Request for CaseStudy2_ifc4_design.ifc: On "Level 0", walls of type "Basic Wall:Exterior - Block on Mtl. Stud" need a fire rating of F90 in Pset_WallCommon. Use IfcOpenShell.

First a look at what the model holds.

```python
import ifcopenshell
import ifcopenshell.util.element

model = ifcopenshell.open("CaseStudy2_ifc4_design.ifc")
print(model.schema)
storey = next(s for s in model.by_type("IfcBuildingStorey") if s.Name == "Level 0")
walls = [e for e in ifcopenshell.util.element.get_decomposition(storey) if e.is_a("IfcWall")]
seen = {}
for e in walls:
    element_type = ifcopenshell.util.element.get_type(e)
    key = (element_type.Name if element_type != e and element_type else None, ifcopenshell.util.element.get_pset(e, "Pset_WallCommon", "FireRating"))
    seen[key] = seen.get(key, 0) + 1
for (name, value), count in sorted(seen.items(), key=str):
    print(count, "x", name, "|", value)
```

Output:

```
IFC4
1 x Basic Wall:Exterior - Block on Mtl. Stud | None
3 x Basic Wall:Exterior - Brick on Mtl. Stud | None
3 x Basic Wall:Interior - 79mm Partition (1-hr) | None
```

```python
import ifcopenshell
import ifcopenshell.api.pset
import ifcopenshell.util.element

model = ifcopenshell.open("CaseStudy2_ifc4_design.ifc")

storey = next(s for s in model.by_type("IfcBuildingStorey") if s.Name == "Level 0")
walls = [e for e in ifcopenshell.util.element.get_decomposition(storey) if e.is_a("IfcWall")]

count = 0
for e in walls:
    element_type = ifcopenshell.util.element.get_type(e)
    if element_type in (None, e) or element_type.Name != "Basic Wall:Exterior - Block on Mtl. Stud":
        continue
    # add_pset returns the element's existing set when there is one.
    pset = ifcopenshell.api.pset.add_pset(model, product=e, name="Pset_WallCommon")
    ifcopenshell.api.pset.edit_pset(model, pset=pset, properties={"FireRating": "F90"})
    count += 1

print(count, "walls updated")

model.write("CaseStudy2_ifc4_design_rev.ifc")
```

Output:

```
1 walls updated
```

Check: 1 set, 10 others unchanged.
